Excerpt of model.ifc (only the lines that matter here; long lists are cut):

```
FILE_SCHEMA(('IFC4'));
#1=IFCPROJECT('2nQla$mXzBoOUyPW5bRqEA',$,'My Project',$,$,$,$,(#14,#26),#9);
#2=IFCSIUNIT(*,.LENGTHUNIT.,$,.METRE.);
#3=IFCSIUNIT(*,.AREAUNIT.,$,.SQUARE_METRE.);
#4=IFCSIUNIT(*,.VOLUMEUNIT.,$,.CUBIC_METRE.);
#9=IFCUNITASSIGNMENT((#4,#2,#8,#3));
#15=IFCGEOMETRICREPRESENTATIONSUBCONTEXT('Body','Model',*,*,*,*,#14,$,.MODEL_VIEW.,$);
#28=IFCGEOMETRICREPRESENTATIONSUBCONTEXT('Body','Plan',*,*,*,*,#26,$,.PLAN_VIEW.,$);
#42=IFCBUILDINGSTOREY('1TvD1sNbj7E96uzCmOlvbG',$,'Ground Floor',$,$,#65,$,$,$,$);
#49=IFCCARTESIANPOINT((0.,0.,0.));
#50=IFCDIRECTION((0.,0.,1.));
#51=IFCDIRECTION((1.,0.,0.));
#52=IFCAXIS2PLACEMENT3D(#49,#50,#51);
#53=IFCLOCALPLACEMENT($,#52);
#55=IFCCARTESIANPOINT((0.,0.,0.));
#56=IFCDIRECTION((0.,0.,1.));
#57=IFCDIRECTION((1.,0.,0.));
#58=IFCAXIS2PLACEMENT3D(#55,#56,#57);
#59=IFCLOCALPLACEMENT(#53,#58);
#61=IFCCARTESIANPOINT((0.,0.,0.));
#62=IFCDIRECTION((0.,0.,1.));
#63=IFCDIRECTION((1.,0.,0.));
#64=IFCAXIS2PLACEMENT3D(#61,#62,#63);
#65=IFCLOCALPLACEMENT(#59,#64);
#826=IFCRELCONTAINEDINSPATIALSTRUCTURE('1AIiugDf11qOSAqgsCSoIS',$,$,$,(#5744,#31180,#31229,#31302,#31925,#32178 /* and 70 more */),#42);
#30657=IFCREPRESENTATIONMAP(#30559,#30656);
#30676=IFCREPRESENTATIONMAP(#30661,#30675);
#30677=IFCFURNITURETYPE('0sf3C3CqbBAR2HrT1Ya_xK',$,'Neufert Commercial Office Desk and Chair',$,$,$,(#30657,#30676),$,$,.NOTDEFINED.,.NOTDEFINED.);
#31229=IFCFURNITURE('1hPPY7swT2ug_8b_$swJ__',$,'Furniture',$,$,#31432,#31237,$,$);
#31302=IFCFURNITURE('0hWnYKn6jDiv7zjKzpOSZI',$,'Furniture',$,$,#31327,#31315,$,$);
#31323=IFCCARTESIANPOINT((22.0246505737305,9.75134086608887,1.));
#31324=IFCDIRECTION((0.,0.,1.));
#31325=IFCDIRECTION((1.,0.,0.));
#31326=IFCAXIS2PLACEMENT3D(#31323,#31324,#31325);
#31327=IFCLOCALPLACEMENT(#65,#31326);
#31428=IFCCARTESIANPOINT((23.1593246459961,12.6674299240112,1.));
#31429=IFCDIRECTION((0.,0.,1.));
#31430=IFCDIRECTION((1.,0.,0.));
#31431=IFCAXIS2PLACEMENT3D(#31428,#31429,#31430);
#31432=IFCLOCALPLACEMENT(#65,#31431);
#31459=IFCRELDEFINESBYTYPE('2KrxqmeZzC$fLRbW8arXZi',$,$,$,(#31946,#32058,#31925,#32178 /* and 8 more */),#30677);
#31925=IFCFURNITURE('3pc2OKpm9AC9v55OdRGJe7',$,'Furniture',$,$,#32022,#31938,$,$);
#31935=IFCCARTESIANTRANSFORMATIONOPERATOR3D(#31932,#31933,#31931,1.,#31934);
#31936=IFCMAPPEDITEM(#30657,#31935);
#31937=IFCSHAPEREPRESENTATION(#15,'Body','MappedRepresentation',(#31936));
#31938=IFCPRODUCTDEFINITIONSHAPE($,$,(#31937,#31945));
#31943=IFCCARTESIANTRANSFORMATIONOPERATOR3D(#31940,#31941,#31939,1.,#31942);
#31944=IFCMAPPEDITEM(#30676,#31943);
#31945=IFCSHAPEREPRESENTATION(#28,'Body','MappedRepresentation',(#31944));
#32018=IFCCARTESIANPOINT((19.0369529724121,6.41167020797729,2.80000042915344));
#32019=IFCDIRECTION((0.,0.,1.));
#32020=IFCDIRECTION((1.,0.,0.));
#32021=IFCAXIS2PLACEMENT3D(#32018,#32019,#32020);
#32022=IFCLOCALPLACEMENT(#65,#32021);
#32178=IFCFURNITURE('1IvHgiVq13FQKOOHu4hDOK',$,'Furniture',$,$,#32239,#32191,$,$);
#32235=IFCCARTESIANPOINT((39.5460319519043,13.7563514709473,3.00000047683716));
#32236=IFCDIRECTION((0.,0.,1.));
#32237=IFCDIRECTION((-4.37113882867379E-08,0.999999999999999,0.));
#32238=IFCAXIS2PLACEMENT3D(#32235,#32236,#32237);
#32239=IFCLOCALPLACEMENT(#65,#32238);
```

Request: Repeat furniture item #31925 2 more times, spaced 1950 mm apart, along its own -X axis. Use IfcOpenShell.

```python
import ifcopenshell
import ifcopenshell.api.geometry
import ifcopenshell.api.root
import ifcopenshell.util.element
import ifcopenshell.util.placement
import ifcopenshell.util.unit

model = ifcopenshell.open("model.ifc")
unit_scale = ifcopenshell.util.unit.calculate_unit_scale(model)

source = model.by_id(31925)
base = ifcopenshell.util.placement.get_local_placement(source.ObjectPlacement)
step = -base[:3, 0] * 1.95 / unit_scale

for i in range(1, 3):
    copy = ifcopenshell.api.root.copy_class(model, product=source)
    copy.Representation = ifcopenshell.util.element.copy_deep(
        model, source.Representation, exclude=["IfcGeometricRepresentationContext", "IfcRepresentationMap"]
    )
    matrix = base.copy()
    matrix[:3, 3] += i * step
    print("added at", matrix[:3, 3].round(3) + 0.0)
    ifcopenshell.api.geometry.edit_object_placement(model, product=copy, matrix=matrix, is_si=False)

model.write("model_edited.ifc")
```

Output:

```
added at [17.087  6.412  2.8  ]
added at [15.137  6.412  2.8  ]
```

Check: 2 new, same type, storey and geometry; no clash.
